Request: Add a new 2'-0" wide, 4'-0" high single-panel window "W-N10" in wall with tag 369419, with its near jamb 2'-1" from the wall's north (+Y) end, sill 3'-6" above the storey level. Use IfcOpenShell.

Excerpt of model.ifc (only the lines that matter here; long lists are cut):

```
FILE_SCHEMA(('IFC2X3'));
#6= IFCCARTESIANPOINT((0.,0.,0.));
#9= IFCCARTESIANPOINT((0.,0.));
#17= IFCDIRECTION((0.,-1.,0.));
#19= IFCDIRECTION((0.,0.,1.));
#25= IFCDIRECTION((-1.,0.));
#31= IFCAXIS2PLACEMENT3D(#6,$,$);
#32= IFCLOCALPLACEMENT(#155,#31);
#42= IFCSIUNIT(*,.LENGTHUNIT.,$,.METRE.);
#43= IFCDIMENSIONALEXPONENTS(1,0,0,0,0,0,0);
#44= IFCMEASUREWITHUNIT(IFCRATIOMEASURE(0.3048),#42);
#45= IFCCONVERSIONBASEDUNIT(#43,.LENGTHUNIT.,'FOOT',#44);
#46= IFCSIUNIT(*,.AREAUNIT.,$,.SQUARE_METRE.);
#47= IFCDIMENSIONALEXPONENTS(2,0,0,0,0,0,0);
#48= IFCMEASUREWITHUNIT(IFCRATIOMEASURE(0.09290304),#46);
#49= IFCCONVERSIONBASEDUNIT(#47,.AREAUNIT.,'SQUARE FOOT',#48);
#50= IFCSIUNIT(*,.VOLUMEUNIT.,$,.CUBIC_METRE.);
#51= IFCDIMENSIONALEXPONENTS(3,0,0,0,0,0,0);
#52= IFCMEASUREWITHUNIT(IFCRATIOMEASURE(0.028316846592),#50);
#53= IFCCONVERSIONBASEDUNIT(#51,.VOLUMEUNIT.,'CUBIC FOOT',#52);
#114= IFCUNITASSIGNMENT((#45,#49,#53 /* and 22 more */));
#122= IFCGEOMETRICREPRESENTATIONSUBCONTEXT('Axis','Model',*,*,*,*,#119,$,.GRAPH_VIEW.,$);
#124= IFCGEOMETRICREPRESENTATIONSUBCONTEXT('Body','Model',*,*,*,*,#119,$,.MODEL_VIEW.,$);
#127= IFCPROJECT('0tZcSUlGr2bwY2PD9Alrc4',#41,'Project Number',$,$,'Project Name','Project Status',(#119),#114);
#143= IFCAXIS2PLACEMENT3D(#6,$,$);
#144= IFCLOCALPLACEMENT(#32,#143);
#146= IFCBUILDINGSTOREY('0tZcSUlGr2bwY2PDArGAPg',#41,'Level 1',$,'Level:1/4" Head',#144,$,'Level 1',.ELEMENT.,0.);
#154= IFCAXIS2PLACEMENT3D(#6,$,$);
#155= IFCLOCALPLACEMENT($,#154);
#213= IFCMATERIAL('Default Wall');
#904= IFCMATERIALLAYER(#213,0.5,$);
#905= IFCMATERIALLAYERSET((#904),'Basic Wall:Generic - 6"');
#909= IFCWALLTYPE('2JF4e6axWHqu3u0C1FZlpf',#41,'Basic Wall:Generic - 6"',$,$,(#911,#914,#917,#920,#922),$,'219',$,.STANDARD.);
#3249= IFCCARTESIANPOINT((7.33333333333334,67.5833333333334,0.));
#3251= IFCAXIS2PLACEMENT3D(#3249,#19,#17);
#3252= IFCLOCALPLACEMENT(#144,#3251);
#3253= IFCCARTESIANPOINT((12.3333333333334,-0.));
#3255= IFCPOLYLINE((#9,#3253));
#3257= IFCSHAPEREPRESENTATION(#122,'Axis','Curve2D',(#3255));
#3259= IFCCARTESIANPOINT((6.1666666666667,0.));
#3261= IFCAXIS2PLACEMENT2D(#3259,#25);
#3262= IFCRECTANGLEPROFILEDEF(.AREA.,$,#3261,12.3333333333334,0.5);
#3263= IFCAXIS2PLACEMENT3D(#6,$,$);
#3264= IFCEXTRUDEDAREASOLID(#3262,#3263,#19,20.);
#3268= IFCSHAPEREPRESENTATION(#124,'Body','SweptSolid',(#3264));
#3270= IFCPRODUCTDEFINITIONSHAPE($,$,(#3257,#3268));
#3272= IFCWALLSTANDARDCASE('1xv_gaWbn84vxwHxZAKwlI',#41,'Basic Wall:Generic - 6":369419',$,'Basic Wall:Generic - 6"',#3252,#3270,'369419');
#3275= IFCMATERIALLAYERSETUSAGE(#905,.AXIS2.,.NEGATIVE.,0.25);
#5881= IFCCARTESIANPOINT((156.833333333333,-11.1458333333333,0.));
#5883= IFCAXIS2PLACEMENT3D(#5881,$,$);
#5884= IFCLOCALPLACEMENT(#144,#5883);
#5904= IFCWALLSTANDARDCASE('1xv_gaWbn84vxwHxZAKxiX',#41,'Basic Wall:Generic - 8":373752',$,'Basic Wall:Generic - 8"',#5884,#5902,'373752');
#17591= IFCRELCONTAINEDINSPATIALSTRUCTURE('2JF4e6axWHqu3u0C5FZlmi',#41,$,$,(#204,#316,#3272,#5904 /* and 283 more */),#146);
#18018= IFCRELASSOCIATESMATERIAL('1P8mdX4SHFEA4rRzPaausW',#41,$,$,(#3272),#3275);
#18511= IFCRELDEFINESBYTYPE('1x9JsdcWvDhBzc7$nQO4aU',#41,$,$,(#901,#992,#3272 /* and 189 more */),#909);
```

```python
import numpy as np
import ifcopenshell
import ifcopenshell.api.feature
import ifcopenshell.api.geometry
import ifcopenshell.api.root
import ifcopenshell.api.spatial
import ifcopenshell.api.type
import ifcopenshell.geom
import ifcopenshell.util.element
import ifcopenshell.util.placement
import ifcopenshell.util.representation
import ifcopenshell.util.shape
import ifcopenshell.util.unit

model = ifcopenshell.open("model.ifc")
unit_scale = ifcopenshell.util.unit.calculate_unit_scale(model)
settings = ifcopenshell.geom.settings()


def volume(element):
    """Net volume in cubic metres, openings subtracted."""
    shape = ifcopenshell.geom.create_shape(settings, element)
    return ifcopenshell.util.shape.get_volume(shape.geometry)


wall = model.by_id(3272)
storey = ifcopenshell.util.element.get_container(wall, ifc_class="IfcBuildingStorey")
context = ifcopenshell.util.representation.get_context(model, "Model", "Body", "MODEL_VIEW")
before = volume(wall)

width, height, from_end, sill = 0.6096, 1.2192, 0.635, 1.0668  # metres

# The wall runs along its own X axis, and the end named is its -X end.
wall_shape = ifcopenshell.geom.create_shape(settings, wall)
x, y, z = ifcopenshell.util.shape.get_vertices(wall_shape.geometry).T
start = x.min() + from_end
face, thickness = float(y.min()), float(y.max() - y.min())
wall_matrix = ifcopenshell.util.placement.get_local_placement(wall.ObjectPlacement)
level = ifcopenshell.util.placement.get_local_placement(storey.ObjectPlacement)[2, 3]


def in_wall(x, y):
    """Placement at x, y metres in the wall's axes, at sill height."""
    matrix = wall_matrix.copy()
    matrix[:, 3] = wall_matrix @ np.array([x / unit_scale, y / unit_scale, 0.0, 1.0])
    matrix[2, 3] = level + sill / unit_scale
    return matrix


# Opening: a box that overshoots both wall faces by 50 mm.
opening = ifcopenshell.api.root.create_entity(model, ifc_class="IfcOpeningElement")
box = ifcopenshell.api.geometry.add_wall_representation(
    model, context=context, length=width, height=height, thickness=thickness + 0.1
)
ifcopenshell.api.geometry.assign_representation(model, product=opening, representation=box)
ifcopenshell.api.geometry.edit_object_placement(model, product=opening, matrix=in_wall(start, face - 0.05), is_si=False)
ifcopenshell.api.feature.add_feature(model, feature=opening, element=wall)

window = ifcopenshell.api.root.create_entity(model, ifc_class="IfcWindow", name="W-N10")
window.OverallWidth, window.OverallHeight = width / unit_scale, height / unit_scale
body = ifcopenshell.api.geometry.add_window_representation(
    model,
    context=context,
    overall_width=window.OverallWidth,
    overall_height=window.OverallHeight,
    partition_type="SINGLE_PANEL",
)
ifcopenshell.api.geometry.assign_representation(model, product=window, representation=body)
ifcopenshell.api.spatial.assign_container(model, products=[window], relating_structure=storey)
fills = ifcopenshell.api.feature.add_filling(model, opening=opening, element=window)
fills.OwnerHistory = window.OwnerHistory  # required in IFC2X3

# IFC2X3 keeps the operation on the window style.
style = ifcopenshell.api.root.create_entity(model, ifc_class="IfcWindowStyle", name="W-N10")
style.OperationType, style.ConstructionType = "SINGLE_PANEL", "NOTDEFINED"
style.ParameterTakesPrecedence = style.Sizeable = False
ifcopenshell.api.type.assign_type(model, related_objects=[window], relating_type=style)

# Centre the window in the wall's thickness.
ifcopenshell.api.geometry.edit_object_placement(model, product=window, matrix=in_wall(start, face), is_si=False)
window_shape = ifcopenshell.geom.create_shape(settings, window)
depth = ifcopenshell.util.shape.get_vertices(window_shape.geometry)[:, 1]
offset = face + thickness / 2 - (depth.min() + depth.max()) / 2
ifcopenshell.api.geometry.edit_object_placement(model, product=window, matrix=in_wall(start, offset), is_si=False)

after = volume(wall)

print(f"wall volume {before:.3f} -> {after:.3f} m3")

model.write("model_v2.ifc")
```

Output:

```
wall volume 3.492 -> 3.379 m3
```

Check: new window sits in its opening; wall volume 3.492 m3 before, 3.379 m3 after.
